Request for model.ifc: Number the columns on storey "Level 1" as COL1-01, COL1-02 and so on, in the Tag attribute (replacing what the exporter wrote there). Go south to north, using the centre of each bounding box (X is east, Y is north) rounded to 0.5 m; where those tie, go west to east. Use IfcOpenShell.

First a look at what the model holds.

```python
import ifcopenshell
import ifcopenshell.util.element
import ifcopenshell.util.placement

model = ifcopenshell.open("model.ifc")
print(model.schema)
storey = next(s for s in model.by_type("IfcBuildingStorey") if s.Name == "Level 1")
columns = [e for e in ifcopenshell.util.element.get_decomposition(storey) if e.is_a("IfcColumn")]
for e in sorted(columns, key=lambda e: e.id()):
    origin = ifcopenshell.util.placement.get_local_placement(e.ObjectPlacement)[:3, 3]
    print(e.id(), e.Tag, e.Name, origin.round(2) + 0.0, sep=" | ")
```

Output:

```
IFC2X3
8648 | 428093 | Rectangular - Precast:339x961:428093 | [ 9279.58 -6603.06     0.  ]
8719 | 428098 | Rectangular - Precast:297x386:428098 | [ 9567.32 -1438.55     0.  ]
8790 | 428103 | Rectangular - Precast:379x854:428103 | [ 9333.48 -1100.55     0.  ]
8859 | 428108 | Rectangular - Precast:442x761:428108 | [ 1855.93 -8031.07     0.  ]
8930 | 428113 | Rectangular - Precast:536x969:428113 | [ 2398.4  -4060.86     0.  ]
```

```python
import ifcopenshell
import ifcopenshell.geom
import ifcopenshell.util.element
import ifcopenshell.util.shape

model = ifcopenshell.open("model.ifc")
settings = ifcopenshell.geom.settings()
settings.set("use-world-coords", True)


def centre(element):
    shape = ifcopenshell.geom.create_shape(settings, element)
    return ifcopenshell.util.shape.get_bbox_centroid(shape.geometry)


storey = next(s for s in model.by_type("IfcBuildingStorey") if s.Name == "Level 1")
columns = [e for e in ifcopenshell.util.element.get_decomposition(storey) if e.is_a("IfcColumn")]

# Insertion points can sit at a corner or the storey origin, so sort by the geometry (in metres).
centres = {e: centre(e) for e in columns}
columns.sort(key=lambda e: (round(centres[e][1] / 0.5), centres[e][0]))

for i, e in enumerate(columns, start=1):
    number = f"COL1-{i:02d}"
    e.Tag = number
    print(e.id(), number)

model.write("model_rev.ifc")
```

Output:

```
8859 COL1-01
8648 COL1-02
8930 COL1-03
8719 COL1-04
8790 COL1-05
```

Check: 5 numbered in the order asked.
